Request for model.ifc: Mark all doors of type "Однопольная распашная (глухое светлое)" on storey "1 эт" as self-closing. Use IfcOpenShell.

First a look at what the model holds.

```python
import ifcopenshell
import ifcopenshell.util.element

model = ifcopenshell.open("model.ifc")
print(model.schema)
storey = next(s for s in model.by_type("IfcBuildingStorey") if s.Name == "1 эт")
doors = [e for e in ifcopenshell.util.element.get_decomposition(storey) if e.is_a("IfcDoor")]
seen = {}
for e in doors:
    element_type = ifcopenshell.util.element.get_type(e)
    key = (element_type.Name if element_type != e and element_type else None, ifcopenshell.util.element.get_pset(e, "Pset_DoorCommon", "SelfClosing"))
    seen[key] = seen.get(key, 0) + 1
for (name, value), count in sorted(seen.items(), key=str):
    print(count, "x", name, "|", value)
```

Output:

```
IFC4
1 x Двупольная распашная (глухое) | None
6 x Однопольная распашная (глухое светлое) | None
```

```python
import ifcopenshell
import ifcopenshell.api.pset
import ifcopenshell.util.element

model = ifcopenshell.open("model.ifc")

storey = next(s for s in model.by_type("IfcBuildingStorey") if s.Name == "1 эт")
doors = [e for e in ifcopenshell.util.element.get_decomposition(storey) if e.is_a("IfcDoor")]

count = 0
for e in doors:
    element_type = ifcopenshell.util.element.get_type(e)
    if element_type in (None, e) or element_type.Name != "Однопольная распашная (глухое светлое)":
        continue
    # add_pset returns the element's existing set when there is one.
    pset = ifcopenshell.api.pset.add_pset(model, product=e, name="Pset_DoorCommon")
    ifcopenshell.api.pset.edit_pset(model, pset=pset, properties={"SelfClosing": True})
    count += 1

print(count, "doors updated")

model.write("model_edited.ifc")
```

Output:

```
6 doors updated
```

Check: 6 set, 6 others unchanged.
